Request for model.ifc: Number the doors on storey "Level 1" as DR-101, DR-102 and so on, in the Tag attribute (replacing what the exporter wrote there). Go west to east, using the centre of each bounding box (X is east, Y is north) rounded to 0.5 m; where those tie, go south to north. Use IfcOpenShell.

First a look at what the model holds.

```python
import ifcopenshell
import ifcopenshell.util.element
import ifcopenshell.util.placement

model = ifcopenshell.open("model.ifc")
print(model.schema)
storey = next(s for s in model.by_type("IfcBuildingStorey") if s.Name == "Level 1")
doors = [e for e in ifcopenshell.util.element.get_decomposition(storey) if e.is_a("IfcDoor")]
for e in sorted(doors, key=lambda e: e.id()):
    origin = ifcopenshell.util.placement.get_local_placement(e.ObjectPlacement)[:3, 3]
    print(e.id(), e.Tag, e.Name, origin.round(2) + 0.0, sep=" | ")
```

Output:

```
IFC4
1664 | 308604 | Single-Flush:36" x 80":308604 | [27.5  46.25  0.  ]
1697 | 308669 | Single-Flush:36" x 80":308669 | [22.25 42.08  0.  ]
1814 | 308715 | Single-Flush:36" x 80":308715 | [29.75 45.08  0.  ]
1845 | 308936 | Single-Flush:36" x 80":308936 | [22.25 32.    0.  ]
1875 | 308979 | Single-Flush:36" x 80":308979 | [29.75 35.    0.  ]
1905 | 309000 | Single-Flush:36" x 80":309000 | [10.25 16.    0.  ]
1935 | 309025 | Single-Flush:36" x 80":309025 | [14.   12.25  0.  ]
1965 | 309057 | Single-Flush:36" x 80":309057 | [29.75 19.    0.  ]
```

```python
import ifcopenshell
import ifcopenshell.geom
import ifcopenshell.util.element
import ifcopenshell.util.shape

model = ifcopenshell.open("model.ifc")
settings = ifcopenshell.geom.settings()
settings.set("use-world-coords", True)


def centre(element):
    shape = ifcopenshell.geom.create_shape(settings, element)
    return ifcopenshell.util.shape.get_bbox_centroid(shape.geometry)


storey = next(s for s in model.by_type("IfcBuildingStorey") if s.Name == "Level 1")
doors = [e for e in ifcopenshell.util.element.get_decomposition(storey) if e.is_a("IfcDoor")]

# Insertion points can sit at a corner or the storey origin, so sort by the geometry (in metres).
centres = {e: centre(e) for e in doors}
doors.sort(key=lambda e: (round(centres[e][0] / 0.5), centres[e][1]))

for i, e in enumerate(doors, start=1):
    number = f"DR-1{i:02d}"
    e.Tag = number
    print(e.id(), number)

model.write("model_v2.ifc")
```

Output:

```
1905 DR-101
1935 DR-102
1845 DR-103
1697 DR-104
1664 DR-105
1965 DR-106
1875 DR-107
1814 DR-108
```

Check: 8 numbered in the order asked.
